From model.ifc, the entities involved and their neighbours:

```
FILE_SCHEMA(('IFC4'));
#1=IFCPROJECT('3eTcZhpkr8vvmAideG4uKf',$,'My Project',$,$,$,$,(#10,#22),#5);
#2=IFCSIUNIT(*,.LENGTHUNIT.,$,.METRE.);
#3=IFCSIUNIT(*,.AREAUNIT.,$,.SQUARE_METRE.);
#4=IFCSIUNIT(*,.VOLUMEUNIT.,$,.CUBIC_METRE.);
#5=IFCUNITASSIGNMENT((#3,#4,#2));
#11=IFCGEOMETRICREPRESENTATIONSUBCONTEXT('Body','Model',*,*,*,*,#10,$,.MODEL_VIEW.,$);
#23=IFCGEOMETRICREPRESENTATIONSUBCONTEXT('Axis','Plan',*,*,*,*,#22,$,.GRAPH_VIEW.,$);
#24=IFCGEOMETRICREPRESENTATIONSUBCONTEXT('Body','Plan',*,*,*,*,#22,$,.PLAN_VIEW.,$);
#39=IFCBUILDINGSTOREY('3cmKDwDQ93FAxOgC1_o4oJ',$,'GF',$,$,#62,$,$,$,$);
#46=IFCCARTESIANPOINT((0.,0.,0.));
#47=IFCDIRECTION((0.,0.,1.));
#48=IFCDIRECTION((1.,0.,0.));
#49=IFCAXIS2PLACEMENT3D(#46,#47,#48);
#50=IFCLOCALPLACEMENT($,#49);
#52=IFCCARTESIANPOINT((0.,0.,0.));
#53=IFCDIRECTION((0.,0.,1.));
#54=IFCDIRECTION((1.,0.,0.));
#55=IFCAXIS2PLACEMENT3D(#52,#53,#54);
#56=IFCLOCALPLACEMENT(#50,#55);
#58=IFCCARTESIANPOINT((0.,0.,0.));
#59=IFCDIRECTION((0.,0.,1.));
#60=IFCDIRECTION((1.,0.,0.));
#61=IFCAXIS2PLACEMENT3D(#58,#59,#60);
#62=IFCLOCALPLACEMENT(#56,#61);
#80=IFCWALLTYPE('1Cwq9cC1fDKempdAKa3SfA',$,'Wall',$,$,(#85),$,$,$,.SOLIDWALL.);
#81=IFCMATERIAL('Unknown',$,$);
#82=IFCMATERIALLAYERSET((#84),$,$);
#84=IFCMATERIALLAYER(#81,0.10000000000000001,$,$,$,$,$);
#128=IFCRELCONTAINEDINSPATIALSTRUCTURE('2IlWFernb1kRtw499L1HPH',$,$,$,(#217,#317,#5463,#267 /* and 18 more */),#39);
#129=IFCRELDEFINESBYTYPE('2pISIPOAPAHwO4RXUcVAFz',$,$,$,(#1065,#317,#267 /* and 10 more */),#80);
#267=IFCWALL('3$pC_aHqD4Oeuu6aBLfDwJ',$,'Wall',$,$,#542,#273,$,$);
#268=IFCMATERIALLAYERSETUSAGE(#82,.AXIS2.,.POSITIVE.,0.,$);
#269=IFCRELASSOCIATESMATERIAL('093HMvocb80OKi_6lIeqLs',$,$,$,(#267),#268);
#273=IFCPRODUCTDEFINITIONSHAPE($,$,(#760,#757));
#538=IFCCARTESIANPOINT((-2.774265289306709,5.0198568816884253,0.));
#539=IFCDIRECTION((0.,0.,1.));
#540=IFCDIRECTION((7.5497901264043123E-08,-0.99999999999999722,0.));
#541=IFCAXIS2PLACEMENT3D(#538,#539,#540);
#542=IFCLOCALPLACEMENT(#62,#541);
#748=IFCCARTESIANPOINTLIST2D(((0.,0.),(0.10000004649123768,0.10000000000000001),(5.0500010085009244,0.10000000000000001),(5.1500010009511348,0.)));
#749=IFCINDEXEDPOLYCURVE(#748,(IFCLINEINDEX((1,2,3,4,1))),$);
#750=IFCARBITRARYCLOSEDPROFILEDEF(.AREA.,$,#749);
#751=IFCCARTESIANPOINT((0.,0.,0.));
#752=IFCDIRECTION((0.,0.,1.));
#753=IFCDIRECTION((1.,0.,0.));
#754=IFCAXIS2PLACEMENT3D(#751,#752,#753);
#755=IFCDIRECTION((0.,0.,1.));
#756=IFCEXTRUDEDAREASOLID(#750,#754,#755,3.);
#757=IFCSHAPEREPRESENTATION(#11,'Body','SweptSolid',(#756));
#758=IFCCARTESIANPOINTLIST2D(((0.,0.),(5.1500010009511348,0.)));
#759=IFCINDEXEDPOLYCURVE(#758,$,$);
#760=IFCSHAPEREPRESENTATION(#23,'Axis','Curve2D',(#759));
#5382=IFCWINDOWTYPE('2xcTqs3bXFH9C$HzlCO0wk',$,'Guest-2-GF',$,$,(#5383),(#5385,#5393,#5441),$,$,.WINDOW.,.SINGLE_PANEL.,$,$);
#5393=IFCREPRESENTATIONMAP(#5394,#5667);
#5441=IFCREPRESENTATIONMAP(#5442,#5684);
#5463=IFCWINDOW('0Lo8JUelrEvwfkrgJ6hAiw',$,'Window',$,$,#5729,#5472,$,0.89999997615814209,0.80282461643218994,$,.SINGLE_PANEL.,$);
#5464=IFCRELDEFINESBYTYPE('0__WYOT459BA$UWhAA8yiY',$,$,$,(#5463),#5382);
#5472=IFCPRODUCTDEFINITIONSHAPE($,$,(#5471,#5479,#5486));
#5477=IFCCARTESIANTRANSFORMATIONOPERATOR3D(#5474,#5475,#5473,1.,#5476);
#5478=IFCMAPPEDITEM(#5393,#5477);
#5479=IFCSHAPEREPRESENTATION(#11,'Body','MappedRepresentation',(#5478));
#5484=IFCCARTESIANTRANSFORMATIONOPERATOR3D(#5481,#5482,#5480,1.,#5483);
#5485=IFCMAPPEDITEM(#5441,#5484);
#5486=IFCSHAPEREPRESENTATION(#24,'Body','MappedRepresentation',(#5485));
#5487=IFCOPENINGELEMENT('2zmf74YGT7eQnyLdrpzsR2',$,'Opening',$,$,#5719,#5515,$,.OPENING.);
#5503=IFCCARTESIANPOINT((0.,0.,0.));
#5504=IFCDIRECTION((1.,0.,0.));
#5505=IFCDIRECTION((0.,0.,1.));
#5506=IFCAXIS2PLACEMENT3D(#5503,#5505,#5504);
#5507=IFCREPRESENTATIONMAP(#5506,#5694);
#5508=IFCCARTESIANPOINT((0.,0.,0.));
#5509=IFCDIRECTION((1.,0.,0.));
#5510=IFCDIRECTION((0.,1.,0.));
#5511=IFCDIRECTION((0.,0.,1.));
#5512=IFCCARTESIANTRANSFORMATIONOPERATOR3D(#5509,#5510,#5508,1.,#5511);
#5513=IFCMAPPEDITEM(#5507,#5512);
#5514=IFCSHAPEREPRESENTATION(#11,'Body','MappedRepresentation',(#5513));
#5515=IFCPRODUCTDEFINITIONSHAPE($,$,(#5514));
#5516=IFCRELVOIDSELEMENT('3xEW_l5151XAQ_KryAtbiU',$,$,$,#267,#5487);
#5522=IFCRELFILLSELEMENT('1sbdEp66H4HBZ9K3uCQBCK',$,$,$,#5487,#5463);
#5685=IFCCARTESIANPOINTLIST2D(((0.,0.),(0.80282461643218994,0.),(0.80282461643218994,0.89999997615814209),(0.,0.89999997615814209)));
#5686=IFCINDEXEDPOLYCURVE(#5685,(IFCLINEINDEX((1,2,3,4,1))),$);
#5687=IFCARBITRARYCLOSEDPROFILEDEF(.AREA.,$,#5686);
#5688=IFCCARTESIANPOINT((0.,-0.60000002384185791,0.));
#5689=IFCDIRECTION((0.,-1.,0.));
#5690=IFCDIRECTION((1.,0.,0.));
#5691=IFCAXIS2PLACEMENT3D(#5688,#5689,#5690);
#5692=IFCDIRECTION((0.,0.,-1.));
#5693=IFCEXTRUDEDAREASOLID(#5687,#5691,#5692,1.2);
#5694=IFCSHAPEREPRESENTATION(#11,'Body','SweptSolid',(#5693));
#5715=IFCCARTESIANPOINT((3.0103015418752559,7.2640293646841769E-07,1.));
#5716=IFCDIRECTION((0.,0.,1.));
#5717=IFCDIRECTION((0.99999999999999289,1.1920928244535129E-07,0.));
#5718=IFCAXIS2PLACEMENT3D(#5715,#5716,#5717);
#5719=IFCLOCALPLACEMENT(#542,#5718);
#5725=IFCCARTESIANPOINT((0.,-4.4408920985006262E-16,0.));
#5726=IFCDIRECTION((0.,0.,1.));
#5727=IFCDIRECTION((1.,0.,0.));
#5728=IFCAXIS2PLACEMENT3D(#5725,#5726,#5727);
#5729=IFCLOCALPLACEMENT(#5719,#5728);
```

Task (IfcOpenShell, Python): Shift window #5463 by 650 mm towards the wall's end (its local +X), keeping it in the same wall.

```python
import ifcopenshell
import ifcopenshell.api.geometry
import ifcopenshell.util.placement
import ifcopenshell.util.unit

model = ifcopenshell.open("model.ifc")
unit_scale = ifcopenshell.util.unit.calculate_unit_scale(model)

window = model.by_id(5463)
opening = window.FillsVoids[0].RelatingOpeningElement
wall = opening.VoidsElements[0].RelatingBuildingElement

wall_matrix = ifcopenshell.util.placement.get_local_placement(wall.ObjectPlacement)
shift = wall_matrix[:3, 0] * 0.65 / unit_scale
before = ifcopenshell.util.placement.get_local_placement(window.ObjectPlacement)[:3, 3].copy()

# The window is placed relative to its opening, so it follows when the opening moves.
matrix = ifcopenshell.util.placement.get_local_placement(opening.ObjectPlacement)
matrix[:3, 3] += shift
ifcopenshell.api.geometry.edit_object_placement(
    model, product=opening, matrix=matrix, is_si=False, should_transform_children=True
)

after = ifcopenshell.util.placement.get_local_placement(window.ObjectPlacement)[:3, 3]
print("window moved by", (after - before).round(3) + 0.0)

model.write("model_edited.ifc")
```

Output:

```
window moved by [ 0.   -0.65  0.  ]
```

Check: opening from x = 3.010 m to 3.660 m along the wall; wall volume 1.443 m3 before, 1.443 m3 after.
